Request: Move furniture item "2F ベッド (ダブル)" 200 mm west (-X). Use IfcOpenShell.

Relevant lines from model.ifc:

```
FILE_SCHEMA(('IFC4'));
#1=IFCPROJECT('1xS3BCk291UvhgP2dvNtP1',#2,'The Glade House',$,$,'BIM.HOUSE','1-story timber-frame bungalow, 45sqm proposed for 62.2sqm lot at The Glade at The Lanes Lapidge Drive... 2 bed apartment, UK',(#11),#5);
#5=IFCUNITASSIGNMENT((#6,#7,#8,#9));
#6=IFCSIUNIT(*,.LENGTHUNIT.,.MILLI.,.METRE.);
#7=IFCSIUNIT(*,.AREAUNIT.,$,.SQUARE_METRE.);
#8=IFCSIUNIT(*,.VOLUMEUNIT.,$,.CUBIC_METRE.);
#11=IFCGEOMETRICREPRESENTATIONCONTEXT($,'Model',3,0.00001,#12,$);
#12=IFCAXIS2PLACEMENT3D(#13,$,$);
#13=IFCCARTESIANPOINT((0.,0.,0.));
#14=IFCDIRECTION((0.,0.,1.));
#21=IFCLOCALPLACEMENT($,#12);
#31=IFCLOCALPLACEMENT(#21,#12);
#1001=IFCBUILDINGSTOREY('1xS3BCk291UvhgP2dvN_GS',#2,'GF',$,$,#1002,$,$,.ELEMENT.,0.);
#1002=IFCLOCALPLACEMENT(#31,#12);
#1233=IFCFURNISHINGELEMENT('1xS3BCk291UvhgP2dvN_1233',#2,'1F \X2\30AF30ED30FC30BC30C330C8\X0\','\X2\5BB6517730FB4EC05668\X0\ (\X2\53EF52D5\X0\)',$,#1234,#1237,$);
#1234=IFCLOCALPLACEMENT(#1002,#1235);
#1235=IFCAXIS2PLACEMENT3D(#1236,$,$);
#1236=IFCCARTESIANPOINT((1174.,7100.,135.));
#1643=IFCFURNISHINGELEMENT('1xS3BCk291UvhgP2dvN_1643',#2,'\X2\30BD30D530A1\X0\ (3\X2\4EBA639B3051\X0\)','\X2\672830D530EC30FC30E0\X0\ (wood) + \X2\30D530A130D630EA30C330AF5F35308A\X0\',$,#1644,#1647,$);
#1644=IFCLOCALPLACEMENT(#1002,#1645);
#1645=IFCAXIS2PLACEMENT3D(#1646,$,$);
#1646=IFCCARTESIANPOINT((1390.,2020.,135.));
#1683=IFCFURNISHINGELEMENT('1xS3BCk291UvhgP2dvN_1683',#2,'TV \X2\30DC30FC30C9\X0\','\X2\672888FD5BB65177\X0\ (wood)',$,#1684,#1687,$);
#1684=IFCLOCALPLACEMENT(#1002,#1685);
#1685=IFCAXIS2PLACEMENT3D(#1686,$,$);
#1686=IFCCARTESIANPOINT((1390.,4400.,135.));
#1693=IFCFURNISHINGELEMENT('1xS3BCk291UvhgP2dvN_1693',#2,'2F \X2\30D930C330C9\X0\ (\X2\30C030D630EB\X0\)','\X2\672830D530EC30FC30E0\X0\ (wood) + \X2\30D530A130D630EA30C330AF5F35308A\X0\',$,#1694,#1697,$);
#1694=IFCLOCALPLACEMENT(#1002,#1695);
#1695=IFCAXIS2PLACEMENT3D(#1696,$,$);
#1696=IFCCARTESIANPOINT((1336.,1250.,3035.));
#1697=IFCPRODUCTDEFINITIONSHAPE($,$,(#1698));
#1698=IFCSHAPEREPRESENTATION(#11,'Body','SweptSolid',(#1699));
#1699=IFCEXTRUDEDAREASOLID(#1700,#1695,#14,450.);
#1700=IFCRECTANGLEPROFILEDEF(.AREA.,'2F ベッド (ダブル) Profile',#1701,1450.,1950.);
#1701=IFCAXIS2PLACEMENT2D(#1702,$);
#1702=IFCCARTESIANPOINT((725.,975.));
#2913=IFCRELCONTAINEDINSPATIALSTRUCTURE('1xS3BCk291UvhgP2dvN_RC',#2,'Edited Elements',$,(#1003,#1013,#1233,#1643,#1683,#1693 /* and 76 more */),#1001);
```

```python
import ifcopenshell
import ifcopenshell.api.geometry
import ifcopenshell.util.placement
import ifcopenshell.util.unit

model = ifcopenshell.open("model.ifc")
unit_scale = ifcopenshell.util.unit.calculate_unit_scale(model)

item = model.by_guid("1xS3BCk291UvhgP2dvN_1693")
matrix = ifcopenshell.util.placement.get_local_placement(item.ObjectPlacement)
matrix[0, 3] -= 0.2 / unit_scale
ifcopenshell.api.geometry.edit_object_placement(model, product=item, matrix=matrix, is_si=False)

print(ifcopenshell.util.placement.get_local_placement(item.ObjectPlacement).round(3) + 0.0)

model.write("model_rev.ifc")
```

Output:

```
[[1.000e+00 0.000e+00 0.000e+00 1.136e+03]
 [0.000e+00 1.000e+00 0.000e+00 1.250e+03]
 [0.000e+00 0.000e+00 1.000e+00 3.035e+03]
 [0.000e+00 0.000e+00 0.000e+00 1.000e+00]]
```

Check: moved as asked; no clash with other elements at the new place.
